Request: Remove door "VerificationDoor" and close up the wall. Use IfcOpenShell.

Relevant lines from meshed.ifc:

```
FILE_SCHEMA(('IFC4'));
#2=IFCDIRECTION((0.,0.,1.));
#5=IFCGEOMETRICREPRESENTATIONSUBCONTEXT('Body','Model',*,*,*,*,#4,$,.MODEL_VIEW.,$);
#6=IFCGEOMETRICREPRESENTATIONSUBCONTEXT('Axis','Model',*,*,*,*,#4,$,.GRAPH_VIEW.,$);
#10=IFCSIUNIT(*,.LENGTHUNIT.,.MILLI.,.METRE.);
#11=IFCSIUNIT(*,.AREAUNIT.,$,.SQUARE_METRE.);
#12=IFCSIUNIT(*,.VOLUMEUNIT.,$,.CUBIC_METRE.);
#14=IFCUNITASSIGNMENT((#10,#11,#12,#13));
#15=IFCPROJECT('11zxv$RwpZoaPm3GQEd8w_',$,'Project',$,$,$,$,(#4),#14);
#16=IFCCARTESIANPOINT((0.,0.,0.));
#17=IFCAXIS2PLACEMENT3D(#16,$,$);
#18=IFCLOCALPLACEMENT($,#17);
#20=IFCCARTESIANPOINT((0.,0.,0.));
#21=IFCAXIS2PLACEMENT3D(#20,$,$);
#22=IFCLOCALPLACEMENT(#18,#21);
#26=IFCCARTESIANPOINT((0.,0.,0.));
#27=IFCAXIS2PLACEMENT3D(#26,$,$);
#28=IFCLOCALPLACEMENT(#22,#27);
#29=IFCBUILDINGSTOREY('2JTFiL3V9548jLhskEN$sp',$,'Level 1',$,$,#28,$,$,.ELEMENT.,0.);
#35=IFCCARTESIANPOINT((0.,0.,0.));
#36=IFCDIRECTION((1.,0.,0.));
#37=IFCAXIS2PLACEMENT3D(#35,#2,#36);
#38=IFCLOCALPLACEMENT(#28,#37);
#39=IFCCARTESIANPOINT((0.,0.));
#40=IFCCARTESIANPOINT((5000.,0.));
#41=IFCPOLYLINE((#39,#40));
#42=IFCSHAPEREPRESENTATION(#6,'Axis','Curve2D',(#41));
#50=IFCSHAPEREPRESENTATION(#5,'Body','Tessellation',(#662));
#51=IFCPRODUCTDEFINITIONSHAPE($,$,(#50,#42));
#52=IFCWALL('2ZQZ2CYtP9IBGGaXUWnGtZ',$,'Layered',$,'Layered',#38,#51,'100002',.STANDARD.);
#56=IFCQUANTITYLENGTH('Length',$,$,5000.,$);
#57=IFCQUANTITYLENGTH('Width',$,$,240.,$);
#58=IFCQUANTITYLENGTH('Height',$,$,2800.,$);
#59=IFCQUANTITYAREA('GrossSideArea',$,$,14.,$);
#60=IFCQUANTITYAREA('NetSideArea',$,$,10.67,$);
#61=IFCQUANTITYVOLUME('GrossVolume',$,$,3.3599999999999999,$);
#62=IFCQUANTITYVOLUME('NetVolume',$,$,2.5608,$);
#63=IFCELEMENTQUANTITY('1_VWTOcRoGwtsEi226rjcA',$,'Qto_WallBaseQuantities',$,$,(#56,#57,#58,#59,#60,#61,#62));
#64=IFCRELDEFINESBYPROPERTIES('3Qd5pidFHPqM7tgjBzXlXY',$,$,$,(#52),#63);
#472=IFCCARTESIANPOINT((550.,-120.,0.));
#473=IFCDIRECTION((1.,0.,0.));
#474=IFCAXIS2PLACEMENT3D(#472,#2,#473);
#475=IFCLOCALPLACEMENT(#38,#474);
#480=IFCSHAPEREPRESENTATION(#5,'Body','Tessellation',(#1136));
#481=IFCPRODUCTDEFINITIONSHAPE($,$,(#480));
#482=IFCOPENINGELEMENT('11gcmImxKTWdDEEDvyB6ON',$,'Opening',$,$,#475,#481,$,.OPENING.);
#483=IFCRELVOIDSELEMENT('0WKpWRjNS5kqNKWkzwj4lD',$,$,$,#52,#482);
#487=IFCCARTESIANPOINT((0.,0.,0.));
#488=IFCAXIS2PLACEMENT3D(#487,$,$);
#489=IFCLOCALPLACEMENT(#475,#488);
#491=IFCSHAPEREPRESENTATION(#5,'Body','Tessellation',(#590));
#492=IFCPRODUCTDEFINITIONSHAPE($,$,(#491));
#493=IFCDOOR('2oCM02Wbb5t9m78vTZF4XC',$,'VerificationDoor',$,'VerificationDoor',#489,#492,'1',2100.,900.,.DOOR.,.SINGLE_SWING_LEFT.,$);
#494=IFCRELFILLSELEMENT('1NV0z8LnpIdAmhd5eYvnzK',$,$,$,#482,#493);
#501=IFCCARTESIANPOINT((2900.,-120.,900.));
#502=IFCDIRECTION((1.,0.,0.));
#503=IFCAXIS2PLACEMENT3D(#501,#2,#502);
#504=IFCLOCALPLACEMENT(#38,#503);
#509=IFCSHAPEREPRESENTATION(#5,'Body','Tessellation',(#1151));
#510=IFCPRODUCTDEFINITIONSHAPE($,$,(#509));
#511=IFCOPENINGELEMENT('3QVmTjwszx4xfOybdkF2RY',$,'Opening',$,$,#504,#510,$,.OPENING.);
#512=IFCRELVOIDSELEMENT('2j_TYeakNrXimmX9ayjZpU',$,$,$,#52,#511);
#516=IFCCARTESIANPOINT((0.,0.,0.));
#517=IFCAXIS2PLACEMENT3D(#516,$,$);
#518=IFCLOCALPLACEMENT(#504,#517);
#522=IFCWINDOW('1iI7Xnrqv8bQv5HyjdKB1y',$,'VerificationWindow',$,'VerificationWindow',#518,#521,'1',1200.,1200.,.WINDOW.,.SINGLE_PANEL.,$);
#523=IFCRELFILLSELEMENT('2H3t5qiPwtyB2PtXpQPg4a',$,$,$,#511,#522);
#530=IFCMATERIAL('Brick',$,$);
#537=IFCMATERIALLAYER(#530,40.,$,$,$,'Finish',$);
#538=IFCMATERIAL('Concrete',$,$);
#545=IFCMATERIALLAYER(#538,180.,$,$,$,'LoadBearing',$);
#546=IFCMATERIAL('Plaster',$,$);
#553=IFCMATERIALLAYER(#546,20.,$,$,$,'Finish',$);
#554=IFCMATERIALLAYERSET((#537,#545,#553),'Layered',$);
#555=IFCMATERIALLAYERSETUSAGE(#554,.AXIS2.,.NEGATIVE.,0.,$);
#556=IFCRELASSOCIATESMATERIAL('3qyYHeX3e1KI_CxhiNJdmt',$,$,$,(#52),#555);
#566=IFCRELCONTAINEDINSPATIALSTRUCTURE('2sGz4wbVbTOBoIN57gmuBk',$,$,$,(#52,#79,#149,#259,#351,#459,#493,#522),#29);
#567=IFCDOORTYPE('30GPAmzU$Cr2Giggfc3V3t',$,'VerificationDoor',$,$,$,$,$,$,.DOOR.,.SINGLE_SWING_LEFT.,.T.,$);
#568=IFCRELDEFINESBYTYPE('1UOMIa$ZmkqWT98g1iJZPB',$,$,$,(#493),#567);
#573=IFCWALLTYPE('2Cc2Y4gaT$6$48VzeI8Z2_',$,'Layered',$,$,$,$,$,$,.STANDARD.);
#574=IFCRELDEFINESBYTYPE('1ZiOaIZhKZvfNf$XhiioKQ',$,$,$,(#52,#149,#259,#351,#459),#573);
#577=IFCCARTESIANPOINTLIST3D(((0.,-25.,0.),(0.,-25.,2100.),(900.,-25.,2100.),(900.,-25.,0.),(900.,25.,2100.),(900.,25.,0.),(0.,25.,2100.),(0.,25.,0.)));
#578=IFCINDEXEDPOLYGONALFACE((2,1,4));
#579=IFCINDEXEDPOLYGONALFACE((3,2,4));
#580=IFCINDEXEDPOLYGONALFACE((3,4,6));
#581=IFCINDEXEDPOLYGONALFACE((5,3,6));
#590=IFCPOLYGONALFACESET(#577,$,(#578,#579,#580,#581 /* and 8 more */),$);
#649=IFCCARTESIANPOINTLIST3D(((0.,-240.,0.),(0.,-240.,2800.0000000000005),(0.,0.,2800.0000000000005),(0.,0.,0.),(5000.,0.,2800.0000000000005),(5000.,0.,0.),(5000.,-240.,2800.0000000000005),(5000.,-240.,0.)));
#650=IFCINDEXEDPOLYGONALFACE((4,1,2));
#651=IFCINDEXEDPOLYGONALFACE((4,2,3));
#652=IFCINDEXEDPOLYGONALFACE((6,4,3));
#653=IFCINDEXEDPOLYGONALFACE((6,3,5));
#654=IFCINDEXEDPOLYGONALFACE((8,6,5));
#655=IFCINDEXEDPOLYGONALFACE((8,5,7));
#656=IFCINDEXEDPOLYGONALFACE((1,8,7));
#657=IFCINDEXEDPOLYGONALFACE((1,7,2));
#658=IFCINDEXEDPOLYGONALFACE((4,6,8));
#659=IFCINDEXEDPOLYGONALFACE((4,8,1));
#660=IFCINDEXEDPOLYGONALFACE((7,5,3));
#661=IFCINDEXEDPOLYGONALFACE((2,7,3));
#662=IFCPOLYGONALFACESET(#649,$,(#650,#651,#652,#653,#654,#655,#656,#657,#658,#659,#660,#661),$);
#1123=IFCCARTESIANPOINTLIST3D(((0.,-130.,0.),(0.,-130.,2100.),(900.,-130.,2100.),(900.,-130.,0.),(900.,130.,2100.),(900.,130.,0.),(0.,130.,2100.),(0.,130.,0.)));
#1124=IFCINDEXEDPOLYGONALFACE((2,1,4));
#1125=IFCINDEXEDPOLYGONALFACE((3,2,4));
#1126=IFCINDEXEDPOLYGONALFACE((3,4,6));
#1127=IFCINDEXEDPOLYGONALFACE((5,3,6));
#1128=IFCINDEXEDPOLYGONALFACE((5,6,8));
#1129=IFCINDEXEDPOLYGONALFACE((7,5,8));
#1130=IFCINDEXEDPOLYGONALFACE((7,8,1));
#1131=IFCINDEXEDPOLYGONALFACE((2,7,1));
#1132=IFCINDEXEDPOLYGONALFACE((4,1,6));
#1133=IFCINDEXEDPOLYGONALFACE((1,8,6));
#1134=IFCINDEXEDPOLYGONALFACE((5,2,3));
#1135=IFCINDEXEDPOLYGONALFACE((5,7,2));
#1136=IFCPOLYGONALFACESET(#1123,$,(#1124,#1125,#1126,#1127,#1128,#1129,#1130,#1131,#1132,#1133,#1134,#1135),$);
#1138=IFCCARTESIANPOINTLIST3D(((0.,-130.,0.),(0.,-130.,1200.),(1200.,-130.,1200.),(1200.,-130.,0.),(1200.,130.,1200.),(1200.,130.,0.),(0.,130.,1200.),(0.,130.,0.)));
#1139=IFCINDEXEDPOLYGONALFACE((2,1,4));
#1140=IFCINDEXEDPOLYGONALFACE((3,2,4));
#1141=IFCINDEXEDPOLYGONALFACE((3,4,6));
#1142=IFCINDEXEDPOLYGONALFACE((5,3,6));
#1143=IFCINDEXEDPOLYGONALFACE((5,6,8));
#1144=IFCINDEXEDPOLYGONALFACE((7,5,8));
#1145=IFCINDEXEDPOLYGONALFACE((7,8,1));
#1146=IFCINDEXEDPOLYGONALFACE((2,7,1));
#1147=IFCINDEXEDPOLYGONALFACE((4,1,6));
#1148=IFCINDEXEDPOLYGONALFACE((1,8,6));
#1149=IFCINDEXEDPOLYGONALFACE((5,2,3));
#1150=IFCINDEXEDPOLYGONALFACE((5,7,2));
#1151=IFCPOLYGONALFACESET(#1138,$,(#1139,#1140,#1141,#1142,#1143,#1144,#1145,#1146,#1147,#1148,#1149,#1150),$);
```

```python
import ifcopenshell
import ifcopenshell.api.feature
import ifcopenshell.api.pset
import ifcopenshell.api.root
import ifcopenshell.geom
import ifcopenshell.util.element
import ifcopenshell.util.shape
import ifcopenshell.util.unit

model = ifcopenshell.open("meshed.ifc")
area_scale = ifcopenshell.util.unit.calculate_unit_scale(model, "AREAUNIT")
volume_scale = ifcopenshell.util.unit.calculate_unit_scale(model, "VOLUMEUNIT")
settings = ifcopenshell.geom.settings()


def volume(element):
    """Net volume in cubic metres, openings subtracted."""
    shape = ifcopenshell.geom.create_shape(settings, element)
    return ifcopenshell.util.shape.get_volume(shape.geometry)


door = model.by_guid("2oCM02Wbb5t9m78vTZF4XC")
opening = door.FillsVoids[0].RelatingOpeningElement
wall = opening.VoidsElements[0].RelatingBuildingElement
before = volume(wall)

ifcopenshell.api.root.remove_product(model, product=door)
ifcopenshell.api.feature.remove_feature(model, feature=opening)

after = volume(wall)
thickness = 0.24  # wall thickness in metres

# Update the wall's stored quantities.
qto = model.by_id(ifcopenshell.util.element.get_pset(wall, "Qto_WallBaseQuantities", should_inherit=False)["id"])
ifcopenshell.api.pset.edit_qto(model, qto=qto, properties={
    "NetSideArea": after / thickness / area_scale,
    "NetVolume": after / volume_scale,
})

print(f"wall volume {before:.3f} -> {after:.3f} m3")

model.write("meshed_v2.ifc")
```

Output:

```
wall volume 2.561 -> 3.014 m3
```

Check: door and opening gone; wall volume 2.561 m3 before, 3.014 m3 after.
